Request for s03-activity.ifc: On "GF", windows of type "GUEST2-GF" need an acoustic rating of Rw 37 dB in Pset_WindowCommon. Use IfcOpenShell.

First a look at what the model holds.

```python
import ifcopenshell
import ifcopenshell.util.element

model = ifcopenshell.open("s03-activity.ifc")
print(model.schema)
storey = next(s for s in model.by_type("IfcBuildingStorey") if s.Name == "GF")
windows = [e for e in ifcopenshell.util.element.get_decomposition(storey) if e.is_a("IfcWindow")]
seen = {}
for e in windows:
    element_type = ifcopenshell.util.element.get_type(e)
    key = (element_type.Name if element_type != e and element_type else None, ifcopenshell.util.element.get_pset(e, "Pset_WindowCommon", "AcousticRating"))
    seen[key] = seen.get(key, 0) + 1
for (name, value), count in sorted(seen.items(), key=str):
    print(count, "x", name, "|", value)
```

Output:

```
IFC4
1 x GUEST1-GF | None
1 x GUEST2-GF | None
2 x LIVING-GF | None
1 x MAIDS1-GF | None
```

```python
import ifcopenshell
import ifcopenshell.api.pset
import ifcopenshell.util.element

model = ifcopenshell.open("s03-activity.ifc")

storey = next(s for s in model.by_type("IfcBuildingStorey") if s.Name == "GF")
windows = [e for e in ifcopenshell.util.element.get_decomposition(storey) if e.is_a("IfcWindow")]

count = 0
for e in windows:
    element_type = ifcopenshell.util.element.get_type(e)
    if element_type in (None, e) or element_type.Name != "GUEST2-GF":
        continue
    # add_pset returns the element's existing set when there is one.
    pset = ifcopenshell.api.pset.add_pset(model, product=e, name="Pset_WindowCommon")
    ifcopenshell.api.pset.edit_pset(model, pset=pset, properties={"AcousticRating": "Rw 37 dB"})
    count += 1

print(count, "windows updated")

model.write("s03-activity_edited.ifc")
```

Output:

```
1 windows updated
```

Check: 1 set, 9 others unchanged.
